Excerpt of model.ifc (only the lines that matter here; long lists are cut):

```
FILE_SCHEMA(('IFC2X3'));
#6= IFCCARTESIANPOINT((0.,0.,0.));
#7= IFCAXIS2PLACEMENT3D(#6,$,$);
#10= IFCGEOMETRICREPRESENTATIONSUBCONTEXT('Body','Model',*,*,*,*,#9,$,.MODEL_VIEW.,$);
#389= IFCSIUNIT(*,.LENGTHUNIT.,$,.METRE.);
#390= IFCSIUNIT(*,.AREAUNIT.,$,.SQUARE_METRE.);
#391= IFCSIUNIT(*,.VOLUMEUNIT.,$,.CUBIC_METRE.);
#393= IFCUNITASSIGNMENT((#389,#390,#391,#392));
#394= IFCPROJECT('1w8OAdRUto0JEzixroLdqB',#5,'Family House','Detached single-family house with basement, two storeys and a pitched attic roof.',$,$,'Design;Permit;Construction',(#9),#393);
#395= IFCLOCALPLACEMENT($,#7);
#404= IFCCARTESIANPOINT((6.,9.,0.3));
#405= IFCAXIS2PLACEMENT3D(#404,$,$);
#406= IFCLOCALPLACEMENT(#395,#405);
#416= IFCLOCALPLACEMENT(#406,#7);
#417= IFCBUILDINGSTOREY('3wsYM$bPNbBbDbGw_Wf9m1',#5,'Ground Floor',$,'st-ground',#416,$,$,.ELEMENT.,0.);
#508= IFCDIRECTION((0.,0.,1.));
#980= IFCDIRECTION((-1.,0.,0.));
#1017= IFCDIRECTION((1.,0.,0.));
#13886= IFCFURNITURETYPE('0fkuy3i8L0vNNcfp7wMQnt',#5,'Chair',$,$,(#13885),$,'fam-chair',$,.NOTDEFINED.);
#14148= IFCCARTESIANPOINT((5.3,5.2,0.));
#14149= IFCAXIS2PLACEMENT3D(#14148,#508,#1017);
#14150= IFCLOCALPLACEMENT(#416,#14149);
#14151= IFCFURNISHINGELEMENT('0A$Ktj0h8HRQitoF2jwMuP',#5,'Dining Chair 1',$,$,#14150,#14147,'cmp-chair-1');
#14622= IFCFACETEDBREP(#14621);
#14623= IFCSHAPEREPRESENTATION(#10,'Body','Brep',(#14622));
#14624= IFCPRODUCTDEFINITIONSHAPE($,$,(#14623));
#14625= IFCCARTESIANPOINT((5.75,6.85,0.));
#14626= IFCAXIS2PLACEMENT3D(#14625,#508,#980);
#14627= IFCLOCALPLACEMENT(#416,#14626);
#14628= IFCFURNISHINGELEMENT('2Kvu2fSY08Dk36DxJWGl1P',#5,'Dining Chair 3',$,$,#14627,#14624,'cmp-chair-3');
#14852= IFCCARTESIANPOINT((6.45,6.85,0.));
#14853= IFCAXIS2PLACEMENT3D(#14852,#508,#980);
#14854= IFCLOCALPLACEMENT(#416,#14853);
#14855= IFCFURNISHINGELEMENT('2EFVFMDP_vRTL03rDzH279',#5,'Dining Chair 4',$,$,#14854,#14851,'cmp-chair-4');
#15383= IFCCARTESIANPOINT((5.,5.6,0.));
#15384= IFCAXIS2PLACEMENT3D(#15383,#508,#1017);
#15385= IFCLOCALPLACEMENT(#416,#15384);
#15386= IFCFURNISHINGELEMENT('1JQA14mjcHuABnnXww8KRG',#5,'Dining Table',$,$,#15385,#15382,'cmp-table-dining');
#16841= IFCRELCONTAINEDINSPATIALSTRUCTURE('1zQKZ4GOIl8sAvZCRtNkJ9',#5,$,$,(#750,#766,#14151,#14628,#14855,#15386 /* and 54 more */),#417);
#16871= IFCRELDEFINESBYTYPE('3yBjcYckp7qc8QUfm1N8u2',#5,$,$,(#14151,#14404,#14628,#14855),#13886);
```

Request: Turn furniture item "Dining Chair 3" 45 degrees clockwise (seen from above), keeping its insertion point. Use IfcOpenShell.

```python
import ifcopenshell
import ifcopenshell.api.geometry
import ifcopenshell.util.placement

model = ifcopenshell.open("model.ifc")

item = model.by_id(14628)
matrix = ifcopenshell.util.placement.get_local_placement(item.ObjectPlacement)
matrix = matrix @ ifcopenshell.util.placement.rotation(-45, "Z")
ifcopenshell.api.geometry.edit_object_placement(model, product=item, matrix=matrix, is_si=False)

print(ifcopenshell.util.placement.get_local_placement(item.ObjectPlacement).round(3) + 0.0)

model.write("model_v2.ifc")
```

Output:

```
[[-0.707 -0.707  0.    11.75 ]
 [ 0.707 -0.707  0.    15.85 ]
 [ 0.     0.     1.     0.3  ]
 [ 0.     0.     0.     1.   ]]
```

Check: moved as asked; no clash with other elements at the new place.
